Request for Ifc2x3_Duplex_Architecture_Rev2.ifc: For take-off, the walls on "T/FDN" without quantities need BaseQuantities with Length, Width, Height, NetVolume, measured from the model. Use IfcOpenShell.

First a look at what the model holds.

```python
import ifcopenshell
import ifcopenshell.util.element
import ifcopenshell.util.unit

model = ifcopenshell.open("Ifc2x3_Duplex_Architecture_Rev2.ifc")
print(model.schema)
for unit_type in ("LENGTHUNIT", "AREAUNIT", "VOLUMEUNIT"):
    print(unit_type, ifcopenshell.util.unit.calculate_unit_scale(model, unit_type))
storey = next(s for s in model.by_type("IfcBuildingStorey") if s.Name == "T/FDN")
walls = [e for e in ifcopenshell.util.element.get_decomposition(storey) if e.is_a("IfcWall")]
for e in sorted(walls, key=lambda e: e.id()):
    print(e.id(), e.is_a(), e.Name, list(ifcopenshell.util.element.get_psets(e, qtos_only=True)), sep=" | ")
```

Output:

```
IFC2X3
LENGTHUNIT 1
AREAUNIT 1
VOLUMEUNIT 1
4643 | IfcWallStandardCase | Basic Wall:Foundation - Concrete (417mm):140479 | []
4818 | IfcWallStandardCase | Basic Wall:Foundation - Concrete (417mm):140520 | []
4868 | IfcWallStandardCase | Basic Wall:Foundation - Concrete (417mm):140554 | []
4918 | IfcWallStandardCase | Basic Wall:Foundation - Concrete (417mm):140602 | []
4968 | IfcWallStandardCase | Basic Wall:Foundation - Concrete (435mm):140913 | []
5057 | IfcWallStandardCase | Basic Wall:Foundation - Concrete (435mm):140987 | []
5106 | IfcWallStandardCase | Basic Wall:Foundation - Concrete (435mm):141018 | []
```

```python
import ifcopenshell
import ifcopenshell.api.pset
import ifcopenshell.geom
import ifcopenshell.util.element
import ifcopenshell.util.shape
import ifcopenshell.util.unit

model = ifcopenshell.open("Ifc2x3_Duplex_Architecture_Rev2.ifc")
unit_scale = ifcopenshell.util.unit.calculate_unit_scale(model)
volume_scale = ifcopenshell.util.unit.calculate_unit_scale(model, "VOLUMEUNIT")
settings = ifcopenshell.geom.settings()

storey = next(s for s in model.by_type("IfcBuildingStorey") if s.Name == "T/FDN")
walls = [e for e in ifcopenshell.util.element.get_decomposition(storey) if e.is_a("IfcWall")]

for e in sorted(walls, key=lambda e: e.id()):
    if ifcopenshell.util.element.get_psets(e, qtos_only=True, should_inherit=False):
        continue
    # Geometry comes back in metres, in the element's own axes.
    shape = ifcopenshell.geom.create_shape(settings, e)
    values = {
        "Length": ifcopenshell.util.shape.get_x(shape.geometry) / unit_scale,
        "Width": ifcopenshell.util.shape.get_y(shape.geometry) / unit_scale,
        "Height": ifcopenshell.util.shape.get_z(shape.geometry) / unit_scale,
        "NetVolume": ifcopenshell.util.shape.get_volume(shape.geometry) / volume_scale,
    }
    qto = ifcopenshell.api.pset.add_qto(model, product=e, name="BaseQuantities")
    ifcopenshell.api.pset.edit_qto(model, qto=qto, properties=values)
    print(e.id(), {k: round(v, 3) for k, v in values.items()})

model.write("Ifc2x3_Duplex_Architecture_Rev2_updated.ifc")
```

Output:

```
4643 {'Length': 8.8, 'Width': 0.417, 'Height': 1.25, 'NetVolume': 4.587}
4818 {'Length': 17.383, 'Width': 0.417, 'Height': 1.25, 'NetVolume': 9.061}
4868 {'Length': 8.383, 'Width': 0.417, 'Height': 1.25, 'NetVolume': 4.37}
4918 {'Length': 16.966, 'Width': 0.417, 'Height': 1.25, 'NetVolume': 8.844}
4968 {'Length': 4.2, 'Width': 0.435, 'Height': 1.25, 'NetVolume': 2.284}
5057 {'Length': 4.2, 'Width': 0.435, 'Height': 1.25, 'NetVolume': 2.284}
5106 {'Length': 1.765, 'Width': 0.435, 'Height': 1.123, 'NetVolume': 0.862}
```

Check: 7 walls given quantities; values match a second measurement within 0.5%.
